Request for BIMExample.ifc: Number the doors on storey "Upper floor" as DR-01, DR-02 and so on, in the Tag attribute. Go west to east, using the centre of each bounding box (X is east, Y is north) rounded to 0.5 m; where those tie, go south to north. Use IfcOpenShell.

First a look at what the model holds.

```python
import ifcopenshell
import ifcopenshell.util.element
import ifcopenshell.util.placement

model = ifcopenshell.open("BIMExample.ifc")
print(model.schema)
storey = next(s for s in model.by_type("IfcBuildingStorey") if s.Name == "Upper floor")
doors = [e for e in ifcopenshell.util.element.get_decomposition(storey) if e.is_a("IfcDoor")]
for e in sorted(doors, key=lambda e: e.id()):
    origin = ifcopenshell.util.placement.get_local_placement(e.ObjectPlacement)[:3, 3]
    print(e.id(), e.Tag, e.Name, origin.round(2) + 0.0, sep=" | ")
```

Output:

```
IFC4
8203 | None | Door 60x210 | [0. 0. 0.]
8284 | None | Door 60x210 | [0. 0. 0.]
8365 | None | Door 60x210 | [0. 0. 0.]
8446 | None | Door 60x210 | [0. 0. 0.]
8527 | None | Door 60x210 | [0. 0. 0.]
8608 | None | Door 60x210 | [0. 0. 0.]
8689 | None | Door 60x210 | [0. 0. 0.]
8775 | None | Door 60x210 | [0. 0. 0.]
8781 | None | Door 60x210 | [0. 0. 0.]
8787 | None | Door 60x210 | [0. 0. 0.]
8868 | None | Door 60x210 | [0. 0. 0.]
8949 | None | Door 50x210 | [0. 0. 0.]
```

```python
import ifcopenshell
import ifcopenshell.geom
import ifcopenshell.util.element
import ifcopenshell.util.shape

model = ifcopenshell.open("BIMExample.ifc")
settings = ifcopenshell.geom.settings()
settings.set("use-world-coords", True)


def centre(element):
    shape = ifcopenshell.geom.create_shape(settings, element)
    return ifcopenshell.util.shape.get_bbox_centroid(shape.geometry)


storey = next(s for s in model.by_type("IfcBuildingStorey") if s.Name == "Upper floor")
doors = [e for e in ifcopenshell.util.element.get_decomposition(storey) if e.is_a("IfcDoor")]

# Insertion points can sit at a corner or the storey origin, so sort by the geometry (in metres).
centres = {e: centre(e) for e in doors}
doors.sort(key=lambda e: (round(centres[e][0] / 0.5), centres[e][1]))

for i, e in enumerate(doors, start=1):
    number = f"DR-{i:02d}"
    e.Tag = number
    print(e.id(), number)

model.write("BIMExample_rev.ifc")
```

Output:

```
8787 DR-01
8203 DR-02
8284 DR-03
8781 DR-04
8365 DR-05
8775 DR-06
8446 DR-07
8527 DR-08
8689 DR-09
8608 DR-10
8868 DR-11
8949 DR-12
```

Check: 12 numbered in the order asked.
